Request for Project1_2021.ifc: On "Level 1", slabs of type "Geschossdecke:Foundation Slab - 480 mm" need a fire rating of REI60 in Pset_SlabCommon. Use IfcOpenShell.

First a look at what the model holds.

```python
import ifcopenshell
import ifcopenshell.util.element

model = ifcopenshell.open("Project1_2021.ifc")
print(model.schema)
storey = next(s for s in model.by_type("IfcBuildingStorey") if s.Name == "Level 1")
slabs = [e for e in ifcopenshell.util.element.get_decomposition(storey) if e.is_a("IfcSlab")]
seen = {}
for e in slabs:
    element_type = ifcopenshell.util.element.get_type(e)
    key = (element_type.Name if element_type != e and element_type else None, ifcopenshell.util.element.get_pset(e, "Pset_SlabCommon", "FireRating"))
    seen[key] = seen.get(key, 0) + 1
for (name, value), count in sorted(seen.items(), key=str):
    print(count, "x", name, "|", value)
```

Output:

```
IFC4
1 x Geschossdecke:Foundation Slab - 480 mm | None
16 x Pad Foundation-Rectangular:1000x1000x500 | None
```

```python
import ifcopenshell
import ifcopenshell.api.pset
import ifcopenshell.util.element

model = ifcopenshell.open("Project1_2021.ifc")

storey = next(s for s in model.by_type("IfcBuildingStorey") if s.Name == "Level 1")
slabs = [e for e in ifcopenshell.util.element.get_decomposition(storey) if e.is_a("IfcSlab")]

count = 0
for e in slabs:
    element_type = ifcopenshell.util.element.get_type(e)
    if element_type in (None, e) or element_type.Name != "Geschossdecke:Foundation Slab - 480 mm":
        continue
    # add_pset returns the element's existing set when there is one.
    pset = ifcopenshell.api.pset.add_pset(model, product=e, name="Pset_SlabCommon")
    ifcopenshell.api.pset.edit_pset(model, pset=pset, properties={"FireRating": "REI60"})
    count += 1

print(count, "slabs updated")

model.write("Project1_2021_rev.ifc")
```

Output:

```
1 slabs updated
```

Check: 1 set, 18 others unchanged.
